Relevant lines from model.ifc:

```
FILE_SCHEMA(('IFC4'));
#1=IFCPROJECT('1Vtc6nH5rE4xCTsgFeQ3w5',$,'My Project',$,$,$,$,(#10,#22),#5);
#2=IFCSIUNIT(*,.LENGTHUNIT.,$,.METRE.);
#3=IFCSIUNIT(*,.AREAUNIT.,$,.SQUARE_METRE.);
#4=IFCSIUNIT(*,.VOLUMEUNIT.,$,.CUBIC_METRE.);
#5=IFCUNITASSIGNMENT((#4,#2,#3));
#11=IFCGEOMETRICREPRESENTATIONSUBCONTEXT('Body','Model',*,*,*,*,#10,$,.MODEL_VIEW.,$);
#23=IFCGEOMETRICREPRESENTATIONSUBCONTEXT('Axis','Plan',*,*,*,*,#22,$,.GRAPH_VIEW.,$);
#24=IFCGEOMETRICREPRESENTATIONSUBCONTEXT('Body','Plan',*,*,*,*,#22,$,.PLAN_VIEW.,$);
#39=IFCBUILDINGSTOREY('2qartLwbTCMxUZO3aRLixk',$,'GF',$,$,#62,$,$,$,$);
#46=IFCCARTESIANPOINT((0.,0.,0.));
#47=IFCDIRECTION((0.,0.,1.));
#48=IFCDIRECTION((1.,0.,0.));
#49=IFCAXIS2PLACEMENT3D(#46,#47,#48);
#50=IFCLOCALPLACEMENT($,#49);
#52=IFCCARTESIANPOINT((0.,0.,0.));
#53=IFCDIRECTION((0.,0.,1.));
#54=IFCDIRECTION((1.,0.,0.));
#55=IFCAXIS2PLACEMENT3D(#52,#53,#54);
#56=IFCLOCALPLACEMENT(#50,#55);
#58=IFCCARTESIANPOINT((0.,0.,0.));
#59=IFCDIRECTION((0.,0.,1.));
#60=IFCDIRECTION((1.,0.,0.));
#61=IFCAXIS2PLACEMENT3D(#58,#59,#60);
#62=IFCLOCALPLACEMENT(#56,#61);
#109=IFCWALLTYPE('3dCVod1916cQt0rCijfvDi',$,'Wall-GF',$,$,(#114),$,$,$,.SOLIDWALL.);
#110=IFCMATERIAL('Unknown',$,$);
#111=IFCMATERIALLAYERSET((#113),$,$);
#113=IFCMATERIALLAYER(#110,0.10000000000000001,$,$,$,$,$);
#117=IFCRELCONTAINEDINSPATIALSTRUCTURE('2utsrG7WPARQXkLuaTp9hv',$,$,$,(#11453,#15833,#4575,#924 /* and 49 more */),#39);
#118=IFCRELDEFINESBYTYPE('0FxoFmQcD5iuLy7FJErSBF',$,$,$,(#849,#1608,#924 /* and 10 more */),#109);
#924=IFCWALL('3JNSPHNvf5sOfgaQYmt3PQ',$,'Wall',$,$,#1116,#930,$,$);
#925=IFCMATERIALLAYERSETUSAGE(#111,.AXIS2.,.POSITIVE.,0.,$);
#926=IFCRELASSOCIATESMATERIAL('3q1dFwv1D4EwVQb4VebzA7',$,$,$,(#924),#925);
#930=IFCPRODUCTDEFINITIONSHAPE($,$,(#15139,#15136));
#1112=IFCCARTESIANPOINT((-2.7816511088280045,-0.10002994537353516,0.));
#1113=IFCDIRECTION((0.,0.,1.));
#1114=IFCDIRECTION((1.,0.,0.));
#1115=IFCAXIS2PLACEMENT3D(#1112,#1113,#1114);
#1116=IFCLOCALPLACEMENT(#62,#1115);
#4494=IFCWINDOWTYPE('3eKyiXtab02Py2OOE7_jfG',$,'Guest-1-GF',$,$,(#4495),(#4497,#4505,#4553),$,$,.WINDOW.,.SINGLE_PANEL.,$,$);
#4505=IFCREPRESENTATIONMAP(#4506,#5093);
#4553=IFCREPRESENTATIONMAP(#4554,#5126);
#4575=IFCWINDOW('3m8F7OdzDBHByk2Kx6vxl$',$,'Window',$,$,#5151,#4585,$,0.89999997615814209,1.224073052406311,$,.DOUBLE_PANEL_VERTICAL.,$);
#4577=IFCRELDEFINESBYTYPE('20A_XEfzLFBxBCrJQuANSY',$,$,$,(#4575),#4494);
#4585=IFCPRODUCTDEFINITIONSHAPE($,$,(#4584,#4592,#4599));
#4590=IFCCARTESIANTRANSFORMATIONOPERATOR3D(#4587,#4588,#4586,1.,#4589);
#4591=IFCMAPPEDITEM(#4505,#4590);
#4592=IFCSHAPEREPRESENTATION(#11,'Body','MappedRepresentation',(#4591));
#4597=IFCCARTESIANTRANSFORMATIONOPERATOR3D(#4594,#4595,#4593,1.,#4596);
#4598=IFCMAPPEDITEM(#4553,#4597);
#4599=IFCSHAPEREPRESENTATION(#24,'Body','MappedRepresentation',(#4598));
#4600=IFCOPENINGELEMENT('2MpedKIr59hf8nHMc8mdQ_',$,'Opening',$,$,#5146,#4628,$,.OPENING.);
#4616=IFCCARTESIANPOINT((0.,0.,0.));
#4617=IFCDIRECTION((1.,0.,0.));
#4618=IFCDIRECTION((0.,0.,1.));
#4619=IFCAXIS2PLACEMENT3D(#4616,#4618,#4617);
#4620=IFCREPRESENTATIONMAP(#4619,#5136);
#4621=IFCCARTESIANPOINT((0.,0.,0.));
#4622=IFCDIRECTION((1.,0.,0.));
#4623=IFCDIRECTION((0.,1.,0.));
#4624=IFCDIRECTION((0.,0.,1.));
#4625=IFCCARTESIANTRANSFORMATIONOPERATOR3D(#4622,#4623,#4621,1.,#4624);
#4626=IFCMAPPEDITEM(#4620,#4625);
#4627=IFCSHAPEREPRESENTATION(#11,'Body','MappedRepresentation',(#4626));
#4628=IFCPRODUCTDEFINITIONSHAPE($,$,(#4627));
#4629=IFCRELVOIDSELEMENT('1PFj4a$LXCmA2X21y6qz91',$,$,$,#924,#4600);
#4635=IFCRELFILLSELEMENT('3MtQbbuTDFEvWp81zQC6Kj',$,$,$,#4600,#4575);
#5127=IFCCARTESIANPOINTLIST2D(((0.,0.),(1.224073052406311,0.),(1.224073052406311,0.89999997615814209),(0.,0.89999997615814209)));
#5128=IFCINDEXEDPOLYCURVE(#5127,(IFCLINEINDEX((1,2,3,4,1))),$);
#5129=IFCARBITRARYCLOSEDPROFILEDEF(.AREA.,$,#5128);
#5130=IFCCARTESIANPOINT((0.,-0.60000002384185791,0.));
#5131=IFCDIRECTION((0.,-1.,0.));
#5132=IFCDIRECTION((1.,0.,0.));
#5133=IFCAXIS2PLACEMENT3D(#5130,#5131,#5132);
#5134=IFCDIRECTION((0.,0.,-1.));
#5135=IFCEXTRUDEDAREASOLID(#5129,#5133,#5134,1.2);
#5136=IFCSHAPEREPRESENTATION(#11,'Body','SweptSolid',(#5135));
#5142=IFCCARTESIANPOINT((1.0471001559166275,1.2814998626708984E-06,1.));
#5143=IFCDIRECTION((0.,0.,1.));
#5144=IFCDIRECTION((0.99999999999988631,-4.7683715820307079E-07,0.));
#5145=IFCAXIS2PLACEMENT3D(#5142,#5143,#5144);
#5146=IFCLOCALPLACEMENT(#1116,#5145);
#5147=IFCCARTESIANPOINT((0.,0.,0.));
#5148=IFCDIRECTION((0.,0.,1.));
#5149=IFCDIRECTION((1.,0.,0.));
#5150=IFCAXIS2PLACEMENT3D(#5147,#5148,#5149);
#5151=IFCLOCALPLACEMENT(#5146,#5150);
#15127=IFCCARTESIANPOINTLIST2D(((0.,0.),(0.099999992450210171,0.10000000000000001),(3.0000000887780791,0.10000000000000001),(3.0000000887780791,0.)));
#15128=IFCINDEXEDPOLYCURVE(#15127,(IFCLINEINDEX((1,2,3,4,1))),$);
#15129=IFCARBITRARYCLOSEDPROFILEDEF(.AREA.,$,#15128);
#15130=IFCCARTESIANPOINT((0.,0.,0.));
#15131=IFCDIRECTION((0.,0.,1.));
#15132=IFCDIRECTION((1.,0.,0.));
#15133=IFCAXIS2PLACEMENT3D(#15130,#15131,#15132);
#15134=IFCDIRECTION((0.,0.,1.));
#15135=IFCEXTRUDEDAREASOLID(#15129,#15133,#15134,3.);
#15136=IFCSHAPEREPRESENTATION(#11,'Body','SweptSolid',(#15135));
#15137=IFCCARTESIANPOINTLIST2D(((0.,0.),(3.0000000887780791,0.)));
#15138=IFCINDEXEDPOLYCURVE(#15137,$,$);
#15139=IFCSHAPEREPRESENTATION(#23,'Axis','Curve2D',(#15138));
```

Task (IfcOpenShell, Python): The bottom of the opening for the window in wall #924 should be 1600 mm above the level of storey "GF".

```python
import numpy as np
import ifcopenshell
import ifcopenshell.api.geometry
import ifcopenshell.geom
import ifcopenshell.util.element
import ifcopenshell.util.placement
import ifcopenshell.util.shape
import ifcopenshell.util.unit

model = ifcopenshell.open("model.ifc")
unit_scale = ifcopenshell.util.unit.calculate_unit_scale(model)

window = model.by_guid("3m8F7OdzDBHByk2Kx6vxl$")
opening = window.FillsVoids[0].RelatingOpeningElement
storey = ifcopenshell.util.element.get_container(window, ifc_class="IfcBuildingStorey")
level = ifcopenshell.util.placement.get_local_placement(storey.ObjectPlacement)[2, 3]

# The opening's origin need not be at the sill, so measure its lowest point.
shape = ifcopenshell.geom.create_shape(ifcopenshell.geom.settings(), opening)
bottom = ifcopenshell.util.shape.get_shape_bottom_elevation(shape, shape.geometry) / unit_scale
dz = level + 1.6 - bottom

shift = np.array([0.0, 0.0, dz])
# The window is placed relative to its opening, so it follows when the opening moves.
matrix = ifcopenshell.util.placement.get_local_placement(opening.ObjectPlacement)
matrix[:3, 3] += shift
ifcopenshell.api.geometry.edit_object_placement(
    model, product=opening, matrix=matrix, is_si=False, should_transform_children=True
)

print(f"moved by {dz * unit_scale:+.3f} m")

model.write("model_updated.ifc")
```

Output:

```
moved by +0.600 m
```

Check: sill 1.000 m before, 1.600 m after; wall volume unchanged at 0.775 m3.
